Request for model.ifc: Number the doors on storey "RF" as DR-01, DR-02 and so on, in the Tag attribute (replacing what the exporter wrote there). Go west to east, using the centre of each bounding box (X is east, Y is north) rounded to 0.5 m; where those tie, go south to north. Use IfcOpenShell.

First a look at what the model holds.

```python
import ifcopenshell
import ifcopenshell.util.element
import ifcopenshell.util.placement

model = ifcopenshell.open("model.ifc")
print(model.schema)
storey = next(s for s in model.by_type("IfcBuildingStorey") if s.Name == "RF")
doors = [e for e in ifcopenshell.util.element.get_decomposition(storey) if e.is_a("IfcDoor")]
for e in sorted(doors, key=lambda e: e.id()):
    origin = ifcopenshell.util.placement.get_local_placement(e.ObjectPlacement)[:3, 3]
    print(e.id(), e.Tag, e.Name, origin.round(2) + 0.0, sep=" | ")
```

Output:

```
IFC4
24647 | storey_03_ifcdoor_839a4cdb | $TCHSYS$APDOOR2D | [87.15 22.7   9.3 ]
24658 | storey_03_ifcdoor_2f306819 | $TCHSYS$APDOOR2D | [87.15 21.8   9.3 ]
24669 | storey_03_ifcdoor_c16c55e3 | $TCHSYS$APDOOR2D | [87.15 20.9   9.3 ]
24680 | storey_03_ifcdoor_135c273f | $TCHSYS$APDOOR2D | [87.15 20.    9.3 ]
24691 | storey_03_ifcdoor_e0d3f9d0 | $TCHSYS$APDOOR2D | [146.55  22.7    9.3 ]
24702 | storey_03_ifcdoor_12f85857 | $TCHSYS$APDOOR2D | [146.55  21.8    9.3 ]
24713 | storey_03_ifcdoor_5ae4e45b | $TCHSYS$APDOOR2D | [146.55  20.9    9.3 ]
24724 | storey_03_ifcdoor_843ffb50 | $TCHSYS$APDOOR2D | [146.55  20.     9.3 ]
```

```python
import ifcopenshell
import ifcopenshell.geom
import ifcopenshell.util.element
import ifcopenshell.util.shape

model = ifcopenshell.open("model.ifc")
settings = ifcopenshell.geom.settings()
settings.set("use-world-coords", True)


def centre(element):
    shape = ifcopenshell.geom.create_shape(settings, element)
    return ifcopenshell.util.shape.get_bbox_centroid(shape.geometry)


storey = next(s for s in model.by_type("IfcBuildingStorey") if s.Name == "RF")
doors = [e for e in ifcopenshell.util.element.get_decomposition(storey) if e.is_a("IfcDoor")]

# Insertion points can sit at a corner or the storey origin, so sort by the geometry (in metres).
centres = {e: centre(e) for e in doors}
doors.sort(key=lambda e: (round(centres[e][0] / 0.5), centres[e][1]))

for i, e in enumerate(doors, start=1):
    number = f"DR-{i:02d}"
    e.Tag = number
    print(e.id(), number)

model.write("model_edited.ifc")
```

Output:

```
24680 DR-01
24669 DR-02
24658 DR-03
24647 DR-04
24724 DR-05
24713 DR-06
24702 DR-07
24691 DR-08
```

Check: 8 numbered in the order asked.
